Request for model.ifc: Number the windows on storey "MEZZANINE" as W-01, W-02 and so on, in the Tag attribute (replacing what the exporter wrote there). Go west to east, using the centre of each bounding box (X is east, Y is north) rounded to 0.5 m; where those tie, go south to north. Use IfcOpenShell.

First a look at what the model holds.

```python
import ifcopenshell
import ifcopenshell.util.element
import ifcopenshell.util.placement

model = ifcopenshell.open("model.ifc")
print(model.schema)
storey = next(s for s in model.by_type("IfcBuildingStorey") if s.Name == "MEZZANINE")
windows = [e for e in ifcopenshell.util.element.get_decomposition(storey) if e.is_a("IfcWindow")]
for e in sorted(windows, key=lambda e: e.id()):
    origin = ifcopenshell.util.placement.get_local_placement(e.ObjectPlacement)[:3, 3]
    print(e.id(), e.Tag, e.Name, origin.round(2) + 0.0, sep=" | ")
```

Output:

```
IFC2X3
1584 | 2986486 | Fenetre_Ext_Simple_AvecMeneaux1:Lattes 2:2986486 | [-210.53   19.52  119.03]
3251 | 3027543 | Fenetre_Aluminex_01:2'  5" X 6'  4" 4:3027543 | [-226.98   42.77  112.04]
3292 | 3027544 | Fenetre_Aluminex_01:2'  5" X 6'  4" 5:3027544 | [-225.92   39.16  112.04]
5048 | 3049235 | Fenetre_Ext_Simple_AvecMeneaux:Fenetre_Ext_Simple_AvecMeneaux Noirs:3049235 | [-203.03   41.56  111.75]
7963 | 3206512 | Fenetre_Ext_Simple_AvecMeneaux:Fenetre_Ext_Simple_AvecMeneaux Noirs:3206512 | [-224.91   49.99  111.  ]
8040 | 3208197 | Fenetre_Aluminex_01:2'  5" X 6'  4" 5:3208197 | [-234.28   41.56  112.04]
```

```python
import ifcopenshell
import ifcopenshell.geom
import ifcopenshell.util.element
import ifcopenshell.util.shape

model = ifcopenshell.open("model.ifc")
settings = ifcopenshell.geom.settings()
settings.set("use-world-coords", True)


def centre(element):
    shape = ifcopenshell.geom.create_shape(settings, element)
    return ifcopenshell.util.shape.get_bbox_centroid(shape.geometry)


storey = next(s for s in model.by_type("IfcBuildingStorey") if s.Name == "MEZZANINE")
windows = [e for e in ifcopenshell.util.element.get_decomposition(storey) if e.is_a("IfcWindow")]

# Insertion points can sit at a corner or the storey origin, so sort by the geometry (in metres).
centres = {e: centre(e) for e in windows}
windows.sort(key=lambda e: (round(centres[e][0] / 0.5), centres[e][1]))

for i, e in enumerate(windows, start=1):
    number = f"W-{i:02d}"
    e.Tag = number
    print(e.id(), number)

model.write("model_edited.ifc")
```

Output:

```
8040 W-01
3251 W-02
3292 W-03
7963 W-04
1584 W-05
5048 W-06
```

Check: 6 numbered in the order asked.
